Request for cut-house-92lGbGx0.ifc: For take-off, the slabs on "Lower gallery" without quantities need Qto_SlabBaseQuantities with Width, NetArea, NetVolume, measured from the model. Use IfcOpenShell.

First a look at what the model holds.

```python
import ifcopenshell
import ifcopenshell.util.element
import ifcopenshell.util.unit

model = ifcopenshell.open("cut-house-92lGbGx0.ifc")
print(model.schema)
for unit_type in ("LENGTHUNIT", "AREAUNIT", "VOLUMEUNIT"):
    print(unit_type, ifcopenshell.util.unit.calculate_unit_scale(model, unit_type))
storey = next(s for s in model.by_type("IfcBuildingStorey") if s.Name == "Lower gallery")
slabs = [e for e in ifcopenshell.util.element.get_decomposition(storey) if e.is_a("IfcSlab")]
for e in sorted(slabs, key=lambda e: e.id()):
    print(e.id(), e.is_a(), e.Name, list(ifcopenshell.util.element.get_psets(e, qtos_only=True)), sep=" | ")
```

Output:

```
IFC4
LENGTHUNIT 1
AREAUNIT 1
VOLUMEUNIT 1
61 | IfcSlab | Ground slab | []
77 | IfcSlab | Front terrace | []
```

```python
import ifcopenshell
import ifcopenshell.api.pset
import ifcopenshell.geom
import ifcopenshell.util.element
import ifcopenshell.util.shape
import ifcopenshell.util.unit

model = ifcopenshell.open("cut-house-92lGbGx0.ifc")
unit_scale = ifcopenshell.util.unit.calculate_unit_scale(model)
area_scale = ifcopenshell.util.unit.calculate_unit_scale(model, "AREAUNIT")
volume_scale = ifcopenshell.util.unit.calculate_unit_scale(model, "VOLUMEUNIT")
settings = ifcopenshell.geom.settings()

storey = next(s for s in model.by_type("IfcBuildingStorey") if s.Name == "Lower gallery")
slabs = [e for e in ifcopenshell.util.element.get_decomposition(storey) if e.is_a("IfcSlab")]

for e in sorted(slabs, key=lambda e: e.id()):
    if ifcopenshell.util.element.get_psets(e, qtos_only=True, should_inherit=False):
        continue
    # Geometry comes back in metres, in the element's own axes.
    shape = ifcopenshell.geom.create_shape(settings, e)
    values = {
        "Width": ifcopenshell.util.shape.get_z(shape.geometry) / unit_scale,
        "NetArea": ifcopenshell.util.shape.get_footprint_area(shape.geometry) / area_scale,
        "NetVolume": ifcopenshell.util.shape.get_volume(shape.geometry) / volume_scale,
    }
    qto = ifcopenshell.api.pset.add_qto(model, product=e, name="Qto_SlabBaseQuantities")
    ifcopenshell.api.pset.edit_qto(model, qto=qto, properties=values)
    print(e.id(), {k: round(v, 3) for k, v in values.items()})

model.write("cut-house-92lGbGx0_rev.ifc")
```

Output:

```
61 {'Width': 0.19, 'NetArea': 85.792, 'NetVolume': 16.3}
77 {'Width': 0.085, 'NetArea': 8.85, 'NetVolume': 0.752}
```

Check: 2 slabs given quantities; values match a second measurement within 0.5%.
